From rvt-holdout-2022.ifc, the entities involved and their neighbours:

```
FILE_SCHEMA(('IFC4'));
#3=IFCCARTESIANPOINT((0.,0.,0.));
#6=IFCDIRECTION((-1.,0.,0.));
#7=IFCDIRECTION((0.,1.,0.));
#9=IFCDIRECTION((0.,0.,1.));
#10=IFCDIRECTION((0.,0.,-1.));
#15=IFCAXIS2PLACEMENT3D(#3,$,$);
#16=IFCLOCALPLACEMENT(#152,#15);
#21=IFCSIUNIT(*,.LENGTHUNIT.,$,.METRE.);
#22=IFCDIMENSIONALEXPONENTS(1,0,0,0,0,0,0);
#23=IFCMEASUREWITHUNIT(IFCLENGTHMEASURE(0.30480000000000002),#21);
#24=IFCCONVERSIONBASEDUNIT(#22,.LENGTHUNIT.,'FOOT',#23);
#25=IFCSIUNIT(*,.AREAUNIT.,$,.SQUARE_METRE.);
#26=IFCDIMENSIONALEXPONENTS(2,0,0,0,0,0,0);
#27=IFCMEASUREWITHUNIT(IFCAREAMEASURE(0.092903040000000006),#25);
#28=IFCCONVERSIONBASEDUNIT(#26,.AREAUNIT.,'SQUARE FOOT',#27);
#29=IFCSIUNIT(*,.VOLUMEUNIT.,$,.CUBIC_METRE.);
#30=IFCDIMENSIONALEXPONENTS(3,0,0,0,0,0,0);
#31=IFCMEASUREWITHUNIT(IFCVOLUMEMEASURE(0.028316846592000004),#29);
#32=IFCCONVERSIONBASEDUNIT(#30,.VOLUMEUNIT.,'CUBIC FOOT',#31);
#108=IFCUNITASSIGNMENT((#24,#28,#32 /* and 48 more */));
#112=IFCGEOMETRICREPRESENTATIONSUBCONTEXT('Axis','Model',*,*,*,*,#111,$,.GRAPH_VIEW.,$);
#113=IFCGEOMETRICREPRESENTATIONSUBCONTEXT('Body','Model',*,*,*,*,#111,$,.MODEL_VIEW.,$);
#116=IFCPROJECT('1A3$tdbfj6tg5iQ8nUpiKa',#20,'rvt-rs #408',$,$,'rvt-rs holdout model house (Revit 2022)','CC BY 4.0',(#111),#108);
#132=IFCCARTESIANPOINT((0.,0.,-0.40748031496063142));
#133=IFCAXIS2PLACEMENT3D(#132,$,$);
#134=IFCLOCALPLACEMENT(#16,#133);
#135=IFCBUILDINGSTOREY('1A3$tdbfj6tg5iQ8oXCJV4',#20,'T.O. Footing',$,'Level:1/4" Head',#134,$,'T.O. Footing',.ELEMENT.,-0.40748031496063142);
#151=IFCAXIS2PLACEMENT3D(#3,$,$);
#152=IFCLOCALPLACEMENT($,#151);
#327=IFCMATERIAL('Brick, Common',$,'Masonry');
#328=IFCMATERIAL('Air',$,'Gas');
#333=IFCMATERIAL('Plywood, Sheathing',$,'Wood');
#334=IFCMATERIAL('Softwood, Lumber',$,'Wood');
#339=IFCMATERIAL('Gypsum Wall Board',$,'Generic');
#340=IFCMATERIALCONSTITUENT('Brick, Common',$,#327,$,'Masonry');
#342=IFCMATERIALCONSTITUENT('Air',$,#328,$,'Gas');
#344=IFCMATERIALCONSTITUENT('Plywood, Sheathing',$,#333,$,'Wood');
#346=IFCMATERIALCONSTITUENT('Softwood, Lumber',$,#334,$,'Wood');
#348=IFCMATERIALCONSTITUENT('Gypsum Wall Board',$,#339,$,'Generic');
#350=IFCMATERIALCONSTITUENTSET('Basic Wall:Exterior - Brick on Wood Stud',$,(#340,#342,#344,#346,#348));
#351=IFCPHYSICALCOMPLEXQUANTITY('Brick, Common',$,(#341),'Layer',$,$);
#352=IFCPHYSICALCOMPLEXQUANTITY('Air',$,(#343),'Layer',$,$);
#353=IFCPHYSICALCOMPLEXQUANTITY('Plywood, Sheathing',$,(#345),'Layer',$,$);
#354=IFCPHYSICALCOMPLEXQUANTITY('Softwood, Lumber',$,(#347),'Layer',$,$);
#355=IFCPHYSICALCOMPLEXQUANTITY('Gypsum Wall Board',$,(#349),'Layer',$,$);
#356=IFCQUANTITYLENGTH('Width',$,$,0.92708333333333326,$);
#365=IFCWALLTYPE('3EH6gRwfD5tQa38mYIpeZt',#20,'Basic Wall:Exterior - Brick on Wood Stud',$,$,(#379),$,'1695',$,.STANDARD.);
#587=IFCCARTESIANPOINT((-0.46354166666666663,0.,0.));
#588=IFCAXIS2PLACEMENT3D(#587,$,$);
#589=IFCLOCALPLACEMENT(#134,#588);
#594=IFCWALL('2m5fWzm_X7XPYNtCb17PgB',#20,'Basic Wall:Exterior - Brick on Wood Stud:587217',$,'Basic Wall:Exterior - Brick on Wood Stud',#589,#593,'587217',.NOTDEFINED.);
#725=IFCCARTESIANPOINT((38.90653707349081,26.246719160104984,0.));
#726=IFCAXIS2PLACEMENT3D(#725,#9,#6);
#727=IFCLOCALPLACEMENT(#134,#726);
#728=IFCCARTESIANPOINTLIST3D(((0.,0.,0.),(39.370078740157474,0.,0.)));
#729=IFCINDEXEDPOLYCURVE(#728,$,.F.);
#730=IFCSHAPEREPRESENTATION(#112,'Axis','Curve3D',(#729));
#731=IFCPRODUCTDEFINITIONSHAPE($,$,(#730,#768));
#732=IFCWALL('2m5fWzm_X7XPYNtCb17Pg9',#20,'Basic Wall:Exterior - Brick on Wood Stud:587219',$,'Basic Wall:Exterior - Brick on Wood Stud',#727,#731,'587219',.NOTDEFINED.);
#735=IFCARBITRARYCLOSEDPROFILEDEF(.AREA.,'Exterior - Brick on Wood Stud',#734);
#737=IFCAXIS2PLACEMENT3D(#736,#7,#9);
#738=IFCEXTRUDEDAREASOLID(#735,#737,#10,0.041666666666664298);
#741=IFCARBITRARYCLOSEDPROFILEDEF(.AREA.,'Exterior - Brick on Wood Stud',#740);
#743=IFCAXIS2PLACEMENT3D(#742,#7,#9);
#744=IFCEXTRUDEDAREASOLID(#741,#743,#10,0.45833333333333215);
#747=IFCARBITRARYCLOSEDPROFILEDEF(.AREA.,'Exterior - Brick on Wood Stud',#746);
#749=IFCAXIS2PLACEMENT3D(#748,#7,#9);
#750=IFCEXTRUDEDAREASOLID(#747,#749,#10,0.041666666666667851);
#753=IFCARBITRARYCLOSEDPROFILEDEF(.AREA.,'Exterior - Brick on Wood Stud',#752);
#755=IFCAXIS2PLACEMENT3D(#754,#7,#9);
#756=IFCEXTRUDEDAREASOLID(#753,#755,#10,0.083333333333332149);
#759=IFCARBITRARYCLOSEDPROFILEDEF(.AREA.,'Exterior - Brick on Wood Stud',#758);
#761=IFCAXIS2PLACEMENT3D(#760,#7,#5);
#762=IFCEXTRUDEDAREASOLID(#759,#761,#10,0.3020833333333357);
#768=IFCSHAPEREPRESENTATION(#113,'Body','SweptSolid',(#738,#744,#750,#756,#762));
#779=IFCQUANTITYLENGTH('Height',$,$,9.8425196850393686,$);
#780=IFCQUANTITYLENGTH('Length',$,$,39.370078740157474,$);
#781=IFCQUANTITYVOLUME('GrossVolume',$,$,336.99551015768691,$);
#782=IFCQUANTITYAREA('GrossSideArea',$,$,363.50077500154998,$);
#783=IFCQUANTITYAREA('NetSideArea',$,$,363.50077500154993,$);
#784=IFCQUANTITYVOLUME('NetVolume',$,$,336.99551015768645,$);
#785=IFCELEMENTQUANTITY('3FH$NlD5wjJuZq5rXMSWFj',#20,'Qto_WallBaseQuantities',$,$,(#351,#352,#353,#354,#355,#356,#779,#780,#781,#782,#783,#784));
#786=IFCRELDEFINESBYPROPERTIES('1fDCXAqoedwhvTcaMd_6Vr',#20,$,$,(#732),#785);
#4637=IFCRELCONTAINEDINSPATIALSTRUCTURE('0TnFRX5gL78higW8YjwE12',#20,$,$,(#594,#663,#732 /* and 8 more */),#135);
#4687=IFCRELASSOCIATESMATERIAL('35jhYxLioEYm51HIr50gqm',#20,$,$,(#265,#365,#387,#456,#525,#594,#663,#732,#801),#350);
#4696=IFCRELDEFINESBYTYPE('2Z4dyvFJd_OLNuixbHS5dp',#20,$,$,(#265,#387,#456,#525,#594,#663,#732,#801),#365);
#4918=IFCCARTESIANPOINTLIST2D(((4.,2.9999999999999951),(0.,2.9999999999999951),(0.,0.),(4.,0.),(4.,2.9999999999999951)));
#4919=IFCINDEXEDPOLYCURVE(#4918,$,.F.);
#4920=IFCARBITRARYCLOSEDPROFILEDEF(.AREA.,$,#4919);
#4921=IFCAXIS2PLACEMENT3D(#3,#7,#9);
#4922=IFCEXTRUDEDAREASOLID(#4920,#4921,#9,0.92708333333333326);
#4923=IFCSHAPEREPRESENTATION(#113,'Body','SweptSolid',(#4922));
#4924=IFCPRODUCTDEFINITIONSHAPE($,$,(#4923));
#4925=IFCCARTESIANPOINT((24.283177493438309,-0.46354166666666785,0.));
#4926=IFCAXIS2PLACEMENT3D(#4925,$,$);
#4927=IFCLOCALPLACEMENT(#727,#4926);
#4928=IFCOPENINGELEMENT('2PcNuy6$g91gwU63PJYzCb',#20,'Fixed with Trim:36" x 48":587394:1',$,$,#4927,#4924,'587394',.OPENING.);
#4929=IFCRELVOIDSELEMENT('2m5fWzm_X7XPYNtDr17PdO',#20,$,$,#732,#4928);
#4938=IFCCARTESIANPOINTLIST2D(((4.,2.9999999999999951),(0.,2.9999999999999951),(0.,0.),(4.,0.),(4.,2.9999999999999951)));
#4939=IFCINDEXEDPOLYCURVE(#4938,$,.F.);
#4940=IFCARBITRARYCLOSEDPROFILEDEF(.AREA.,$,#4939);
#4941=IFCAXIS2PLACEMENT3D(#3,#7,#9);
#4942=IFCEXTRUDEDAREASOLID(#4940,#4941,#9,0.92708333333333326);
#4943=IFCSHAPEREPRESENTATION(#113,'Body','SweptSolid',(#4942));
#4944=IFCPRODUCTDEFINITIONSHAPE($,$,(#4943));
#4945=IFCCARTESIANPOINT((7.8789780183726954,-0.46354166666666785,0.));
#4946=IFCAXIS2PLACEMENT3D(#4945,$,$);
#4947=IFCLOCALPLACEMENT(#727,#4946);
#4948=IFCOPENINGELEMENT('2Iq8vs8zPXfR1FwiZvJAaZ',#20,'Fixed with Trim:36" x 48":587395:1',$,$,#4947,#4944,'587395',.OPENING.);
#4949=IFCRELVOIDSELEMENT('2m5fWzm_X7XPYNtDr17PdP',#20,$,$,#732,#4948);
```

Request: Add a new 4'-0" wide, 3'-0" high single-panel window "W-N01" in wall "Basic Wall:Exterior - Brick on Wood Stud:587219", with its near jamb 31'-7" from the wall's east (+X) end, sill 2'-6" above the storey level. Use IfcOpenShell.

```python
import numpy as np
import ifcopenshell
import ifcopenshell.api.feature
import ifcopenshell.api.geometry
import ifcopenshell.api.pset
import ifcopenshell.api.root
import ifcopenshell.api.spatial
import ifcopenshell.geom
import ifcopenshell.util.element
import ifcopenshell.util.placement
import ifcopenshell.util.representation
import ifcopenshell.util.shape
import ifcopenshell.util.unit

model = ifcopenshell.open("rvt-holdout-2022.ifc")
unit_scale = ifcopenshell.util.unit.calculate_unit_scale(model)
area_scale = ifcopenshell.util.unit.calculate_unit_scale(model, "AREAUNIT")
volume_scale = ifcopenshell.util.unit.calculate_unit_scale(model, "VOLUMEUNIT")
settings = ifcopenshell.geom.settings()


def volume(element):
    """Net volume in cubic metres, openings subtracted."""
    shape = ifcopenshell.geom.create_shape(settings, element)
    return ifcopenshell.util.shape.get_volume(shape.geometry)


wall = model.by_guid("2m5fWzm_X7XPYNtCb17Pg9")
storey = ifcopenshell.util.element.get_container(wall, ifc_class="IfcBuildingStorey")
context = ifcopenshell.util.representation.get_context(model, "Model", "Body", "MODEL_VIEW")
before = volume(wall)

width, height, from_end, sill = 1.2192, 0.9144, 9.6266, 0.762  # metres

# The wall runs along its own X axis, and the end named is its -X end.
wall_shape = ifcopenshell.geom.create_shape(settings, wall)
x, y, z = ifcopenshell.util.shape.get_vertices(wall_shape.geometry).T
start = x.min() + from_end
face, thickness = float(y.min()), float(y.max() - y.min())
wall_matrix = ifcopenshell.util.placement.get_local_placement(wall.ObjectPlacement)
level = ifcopenshell.util.placement.get_local_placement(storey.ObjectPlacement)[2, 3]


def in_wall(x, y):
    """Placement at x, y metres in the wall's axes, at sill height."""
    matrix = wall_matrix.copy()
    matrix[:, 3] = wall_matrix @ np.array([x / unit_scale, y / unit_scale, 0.0, 1.0])
    matrix[2, 3] = level + sill / unit_scale
    return matrix


# Opening: a box that overshoots both wall faces by 50 mm.
opening = ifcopenshell.api.root.create_entity(model, ifc_class="IfcOpeningElement", predefined_type="OPENING")
box = ifcopenshell.api.geometry.add_wall_representation(
    model, context=context, length=width, height=height, thickness=thickness + 0.1
)
ifcopenshell.api.geometry.assign_representation(model, product=opening, representation=box)
ifcopenshell.api.geometry.edit_object_placement(model, product=opening, matrix=in_wall(start, face - 0.05), is_si=False)
ifcopenshell.api.feature.add_feature(model, feature=opening, element=wall)

window = ifcopenshell.api.root.create_entity(model, ifc_class="IfcWindow", name="W-N01", predefined_type="WINDOW")
window.OverallWidth, window.OverallHeight = width / unit_scale, height / unit_scale
window.PartitioningType = "SINGLE_PANEL"
body = ifcopenshell.api.geometry.add_window_representation(
    model,
    context=context,
    overall_width=window.OverallWidth,
    overall_height=window.OverallHeight,
    partition_type="SINGLE_PANEL",
)
ifcopenshell.api.geometry.assign_representation(model, product=window, representation=body)
ifcopenshell.api.spatial.assign_container(model, products=[window], relating_structure=storey)
ifcopenshell.api.feature.add_filling(model, opening=opening, element=window)

# Centre the window in the wall's thickness.
ifcopenshell.api.geometry.edit_object_placement(model, product=window, matrix=in_wall(start, face), is_si=False)
window_shape = ifcopenshell.geom.create_shape(settings, window)
depth = ifcopenshell.util.shape.get_vertices(window_shape.geometry)[:, 1]
offset = face + thickness / 2 - (depth.min() + depth.max()) / 2
ifcopenshell.api.geometry.edit_object_placement(model, product=window, matrix=in_wall(start, offset), is_si=False)

after = volume(wall)

# Update the wall's stored quantities.
qto = model.by_id(ifcopenshell.util.element.get_pset(wall, "Qto_WallBaseQuantities", should_inherit=False)["id"])
ifcopenshell.api.pset.edit_qto(model, qto=qto, properties={
    "NetSideArea": after / thickness / area_scale,
    "NetVolume": after / volume_scale,
})

print(f"wall volume {before:.3f} -> {after:.3f} m3")

model.write("rvt-holdout-2022_updated.ifc")
```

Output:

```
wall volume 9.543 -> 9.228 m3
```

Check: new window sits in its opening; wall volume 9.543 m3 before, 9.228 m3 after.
